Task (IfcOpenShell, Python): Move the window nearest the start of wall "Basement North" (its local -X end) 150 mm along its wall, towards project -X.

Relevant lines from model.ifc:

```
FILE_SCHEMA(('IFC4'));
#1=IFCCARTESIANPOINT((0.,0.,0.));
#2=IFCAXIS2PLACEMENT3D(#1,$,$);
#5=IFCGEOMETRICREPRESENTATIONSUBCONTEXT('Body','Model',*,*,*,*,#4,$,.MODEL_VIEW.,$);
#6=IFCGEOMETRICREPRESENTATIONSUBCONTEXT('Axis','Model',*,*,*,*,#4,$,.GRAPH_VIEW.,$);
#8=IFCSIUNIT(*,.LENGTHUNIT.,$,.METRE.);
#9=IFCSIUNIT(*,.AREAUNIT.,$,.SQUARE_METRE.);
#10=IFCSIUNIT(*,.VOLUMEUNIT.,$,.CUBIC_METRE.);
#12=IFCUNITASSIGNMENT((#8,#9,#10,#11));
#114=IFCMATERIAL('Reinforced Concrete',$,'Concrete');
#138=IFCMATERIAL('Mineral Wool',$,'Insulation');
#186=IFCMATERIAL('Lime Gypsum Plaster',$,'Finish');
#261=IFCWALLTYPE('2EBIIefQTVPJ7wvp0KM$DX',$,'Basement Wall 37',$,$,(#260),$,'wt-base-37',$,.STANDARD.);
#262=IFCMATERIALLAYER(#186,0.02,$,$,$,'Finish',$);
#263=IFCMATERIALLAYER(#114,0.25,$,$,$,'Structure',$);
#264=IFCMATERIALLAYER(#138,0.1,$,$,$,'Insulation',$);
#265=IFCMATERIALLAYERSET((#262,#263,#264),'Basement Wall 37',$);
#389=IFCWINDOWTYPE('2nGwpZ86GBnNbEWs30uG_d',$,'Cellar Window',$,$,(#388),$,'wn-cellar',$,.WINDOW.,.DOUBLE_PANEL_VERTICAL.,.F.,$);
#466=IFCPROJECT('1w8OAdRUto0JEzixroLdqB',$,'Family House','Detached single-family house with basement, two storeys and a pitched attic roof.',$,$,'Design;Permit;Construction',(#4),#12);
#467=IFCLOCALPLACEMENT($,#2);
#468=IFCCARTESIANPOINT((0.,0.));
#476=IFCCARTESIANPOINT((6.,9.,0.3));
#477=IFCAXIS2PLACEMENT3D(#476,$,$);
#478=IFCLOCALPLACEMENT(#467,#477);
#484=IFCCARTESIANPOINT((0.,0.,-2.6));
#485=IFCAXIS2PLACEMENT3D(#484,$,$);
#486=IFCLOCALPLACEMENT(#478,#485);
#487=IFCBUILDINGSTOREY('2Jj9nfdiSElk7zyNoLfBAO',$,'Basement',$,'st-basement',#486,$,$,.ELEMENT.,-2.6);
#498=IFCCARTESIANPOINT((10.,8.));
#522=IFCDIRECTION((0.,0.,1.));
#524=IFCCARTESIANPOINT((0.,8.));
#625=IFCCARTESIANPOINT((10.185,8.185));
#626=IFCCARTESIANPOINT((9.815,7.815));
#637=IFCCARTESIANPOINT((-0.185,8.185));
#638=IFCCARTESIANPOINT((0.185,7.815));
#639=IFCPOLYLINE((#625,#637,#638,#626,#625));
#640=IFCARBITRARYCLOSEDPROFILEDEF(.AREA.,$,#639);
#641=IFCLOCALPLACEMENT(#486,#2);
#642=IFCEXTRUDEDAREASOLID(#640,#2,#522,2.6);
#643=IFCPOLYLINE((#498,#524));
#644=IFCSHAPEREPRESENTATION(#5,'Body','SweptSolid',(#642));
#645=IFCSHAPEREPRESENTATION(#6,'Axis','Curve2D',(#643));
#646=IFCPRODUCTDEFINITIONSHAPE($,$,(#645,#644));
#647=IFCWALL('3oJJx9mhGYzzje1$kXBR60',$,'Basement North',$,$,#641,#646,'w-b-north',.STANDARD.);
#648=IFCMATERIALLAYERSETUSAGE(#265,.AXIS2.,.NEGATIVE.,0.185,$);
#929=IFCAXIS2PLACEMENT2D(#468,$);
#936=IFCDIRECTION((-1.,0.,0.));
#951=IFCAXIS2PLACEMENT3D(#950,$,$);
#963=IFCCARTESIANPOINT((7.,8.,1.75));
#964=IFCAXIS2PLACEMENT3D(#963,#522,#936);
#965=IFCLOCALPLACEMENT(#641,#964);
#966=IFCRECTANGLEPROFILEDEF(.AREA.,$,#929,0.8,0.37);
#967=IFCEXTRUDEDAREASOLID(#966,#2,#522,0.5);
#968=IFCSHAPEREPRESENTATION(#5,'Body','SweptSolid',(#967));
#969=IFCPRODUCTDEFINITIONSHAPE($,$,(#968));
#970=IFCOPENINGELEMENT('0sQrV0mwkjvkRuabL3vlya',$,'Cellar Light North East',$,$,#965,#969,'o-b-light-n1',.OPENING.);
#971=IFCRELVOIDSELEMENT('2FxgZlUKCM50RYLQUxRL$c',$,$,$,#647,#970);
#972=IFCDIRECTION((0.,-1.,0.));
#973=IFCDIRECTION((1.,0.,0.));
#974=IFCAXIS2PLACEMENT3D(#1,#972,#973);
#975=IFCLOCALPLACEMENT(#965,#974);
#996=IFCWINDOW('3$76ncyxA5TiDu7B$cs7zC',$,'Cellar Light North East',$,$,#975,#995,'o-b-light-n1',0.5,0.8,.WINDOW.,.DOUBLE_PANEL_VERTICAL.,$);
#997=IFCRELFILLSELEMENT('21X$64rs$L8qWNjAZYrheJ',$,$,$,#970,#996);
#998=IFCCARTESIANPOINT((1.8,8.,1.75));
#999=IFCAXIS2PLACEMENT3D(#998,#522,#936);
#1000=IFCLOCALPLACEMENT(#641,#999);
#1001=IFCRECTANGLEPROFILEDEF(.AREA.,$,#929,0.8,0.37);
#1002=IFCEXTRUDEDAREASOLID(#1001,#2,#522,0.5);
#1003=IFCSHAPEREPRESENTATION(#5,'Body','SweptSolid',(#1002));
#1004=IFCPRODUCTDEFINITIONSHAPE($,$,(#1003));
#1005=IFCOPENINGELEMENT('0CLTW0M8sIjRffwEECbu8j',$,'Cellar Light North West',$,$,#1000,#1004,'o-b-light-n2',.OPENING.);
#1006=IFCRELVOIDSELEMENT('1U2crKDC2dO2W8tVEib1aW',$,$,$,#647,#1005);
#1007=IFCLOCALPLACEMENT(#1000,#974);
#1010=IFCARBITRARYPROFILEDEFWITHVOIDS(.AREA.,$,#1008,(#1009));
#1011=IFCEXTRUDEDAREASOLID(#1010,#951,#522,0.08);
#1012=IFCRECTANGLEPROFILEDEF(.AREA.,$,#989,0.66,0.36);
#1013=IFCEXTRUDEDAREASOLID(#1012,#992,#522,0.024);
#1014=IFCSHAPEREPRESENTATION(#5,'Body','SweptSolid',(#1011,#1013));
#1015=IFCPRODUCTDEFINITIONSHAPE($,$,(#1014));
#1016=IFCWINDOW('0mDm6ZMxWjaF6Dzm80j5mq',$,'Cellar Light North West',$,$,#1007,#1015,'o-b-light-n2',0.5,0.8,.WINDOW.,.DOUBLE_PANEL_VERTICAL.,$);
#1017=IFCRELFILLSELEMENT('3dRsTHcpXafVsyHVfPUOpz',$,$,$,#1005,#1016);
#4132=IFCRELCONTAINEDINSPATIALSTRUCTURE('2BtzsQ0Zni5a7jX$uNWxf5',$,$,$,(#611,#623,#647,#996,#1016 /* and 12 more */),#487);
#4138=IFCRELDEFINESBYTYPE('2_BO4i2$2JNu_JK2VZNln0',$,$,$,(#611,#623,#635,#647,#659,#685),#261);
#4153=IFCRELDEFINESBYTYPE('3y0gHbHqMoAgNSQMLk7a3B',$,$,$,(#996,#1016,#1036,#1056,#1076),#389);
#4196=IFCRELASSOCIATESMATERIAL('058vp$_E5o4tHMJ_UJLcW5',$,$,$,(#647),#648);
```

```python
import ifcopenshell
import ifcopenshell.api.geometry
import ifcopenshell.util.placement

model = ifcopenshell.open("model.ifc")

window = model.by_guid("0mDm6ZMxWjaF6Dzm80j5mq")
opening = window.FillsVoids[0].RelatingOpeningElement
wall = opening.VoidsElements[0].RelatingBuildingElement

wall_matrix = ifcopenshell.util.placement.get_local_placement(wall.ObjectPlacement)
shift = wall_matrix[:3, 0] * -0.15
before = ifcopenshell.util.placement.get_local_placement(window.ObjectPlacement)[:3, 3].copy()

# The window is placed relative to its opening, so it follows when the opening moves.
matrix = ifcopenshell.util.placement.get_local_placement(opening.ObjectPlacement)
matrix[:3, 3] += shift
ifcopenshell.api.geometry.edit_object_placement(
    model, product=opening, matrix=matrix, is_si=False, should_transform_children=True
)

after = ifcopenshell.util.placement.get_local_placement(window.ObjectPlacement)[:3, 3]
print("window moved by", (after - before).round(3) + 0.0)

model.write("model_edited.ifc")
```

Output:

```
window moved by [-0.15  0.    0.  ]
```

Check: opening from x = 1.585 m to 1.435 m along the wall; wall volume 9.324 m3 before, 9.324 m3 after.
